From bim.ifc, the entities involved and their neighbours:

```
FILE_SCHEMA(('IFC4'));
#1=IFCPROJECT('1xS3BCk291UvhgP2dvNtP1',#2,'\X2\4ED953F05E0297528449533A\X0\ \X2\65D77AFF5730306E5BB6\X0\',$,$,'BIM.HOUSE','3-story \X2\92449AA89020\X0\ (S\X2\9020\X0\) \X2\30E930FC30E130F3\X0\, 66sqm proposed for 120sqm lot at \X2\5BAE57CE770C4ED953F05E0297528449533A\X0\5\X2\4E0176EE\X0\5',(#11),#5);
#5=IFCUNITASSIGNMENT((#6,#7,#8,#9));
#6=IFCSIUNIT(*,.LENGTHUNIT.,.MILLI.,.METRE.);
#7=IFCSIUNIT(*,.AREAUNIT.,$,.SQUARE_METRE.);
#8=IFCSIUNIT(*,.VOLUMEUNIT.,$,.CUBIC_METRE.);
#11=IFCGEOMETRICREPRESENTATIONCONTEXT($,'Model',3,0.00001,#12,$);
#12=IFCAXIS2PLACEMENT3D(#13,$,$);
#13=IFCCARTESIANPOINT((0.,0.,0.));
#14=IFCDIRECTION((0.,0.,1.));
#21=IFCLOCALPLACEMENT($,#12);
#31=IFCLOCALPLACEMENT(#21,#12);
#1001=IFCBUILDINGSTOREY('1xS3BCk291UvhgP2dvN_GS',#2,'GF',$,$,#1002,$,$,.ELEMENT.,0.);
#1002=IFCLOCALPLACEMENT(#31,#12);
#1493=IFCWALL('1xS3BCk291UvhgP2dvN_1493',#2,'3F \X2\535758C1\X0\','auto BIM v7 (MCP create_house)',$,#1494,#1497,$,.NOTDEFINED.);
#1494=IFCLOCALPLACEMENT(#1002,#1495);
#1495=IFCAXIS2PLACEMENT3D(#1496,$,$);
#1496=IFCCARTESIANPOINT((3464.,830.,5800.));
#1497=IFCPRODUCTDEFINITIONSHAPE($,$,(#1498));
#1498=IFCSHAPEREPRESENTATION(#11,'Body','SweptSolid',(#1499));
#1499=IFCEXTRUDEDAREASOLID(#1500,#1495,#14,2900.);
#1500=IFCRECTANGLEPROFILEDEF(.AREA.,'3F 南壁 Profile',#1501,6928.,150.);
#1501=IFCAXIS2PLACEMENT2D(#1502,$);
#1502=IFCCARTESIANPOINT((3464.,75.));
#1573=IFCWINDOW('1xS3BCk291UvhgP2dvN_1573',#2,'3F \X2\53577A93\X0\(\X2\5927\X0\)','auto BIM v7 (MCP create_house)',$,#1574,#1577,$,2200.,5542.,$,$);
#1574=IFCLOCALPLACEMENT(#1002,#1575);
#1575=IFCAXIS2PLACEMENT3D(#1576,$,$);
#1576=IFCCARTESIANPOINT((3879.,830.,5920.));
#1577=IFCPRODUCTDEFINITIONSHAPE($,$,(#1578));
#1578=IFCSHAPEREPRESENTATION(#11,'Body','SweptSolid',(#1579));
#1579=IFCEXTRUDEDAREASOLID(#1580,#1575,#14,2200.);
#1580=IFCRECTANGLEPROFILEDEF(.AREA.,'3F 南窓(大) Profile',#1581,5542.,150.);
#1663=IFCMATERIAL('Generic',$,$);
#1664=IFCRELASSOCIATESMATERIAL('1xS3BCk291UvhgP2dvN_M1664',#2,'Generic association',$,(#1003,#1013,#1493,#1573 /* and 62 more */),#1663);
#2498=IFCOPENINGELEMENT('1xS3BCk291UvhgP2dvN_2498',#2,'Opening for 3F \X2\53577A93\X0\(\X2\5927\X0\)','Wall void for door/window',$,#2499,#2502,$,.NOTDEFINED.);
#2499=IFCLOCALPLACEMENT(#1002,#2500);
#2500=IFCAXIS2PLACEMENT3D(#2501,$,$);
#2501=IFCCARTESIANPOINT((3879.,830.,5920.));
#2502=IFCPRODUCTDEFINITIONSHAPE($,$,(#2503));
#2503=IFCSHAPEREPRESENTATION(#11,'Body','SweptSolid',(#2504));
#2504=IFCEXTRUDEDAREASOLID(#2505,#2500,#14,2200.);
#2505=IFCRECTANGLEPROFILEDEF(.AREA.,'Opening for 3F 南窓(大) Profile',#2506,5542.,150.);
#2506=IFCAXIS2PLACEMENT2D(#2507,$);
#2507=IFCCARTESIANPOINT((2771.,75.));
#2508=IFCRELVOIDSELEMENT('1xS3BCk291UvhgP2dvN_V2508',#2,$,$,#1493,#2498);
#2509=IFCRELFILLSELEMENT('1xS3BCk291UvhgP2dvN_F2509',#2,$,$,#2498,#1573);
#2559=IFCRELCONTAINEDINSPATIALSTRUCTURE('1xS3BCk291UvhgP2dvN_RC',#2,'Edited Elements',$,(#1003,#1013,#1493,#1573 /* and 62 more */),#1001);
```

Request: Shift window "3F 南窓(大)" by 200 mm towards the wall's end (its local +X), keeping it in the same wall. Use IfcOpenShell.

```python
import ifcopenshell
import ifcopenshell.api.geometry
import ifcopenshell.util.placement
import ifcopenshell.util.unit

model = ifcopenshell.open("bim.ifc")
unit_scale = ifcopenshell.util.unit.calculate_unit_scale(model)

window = model.by_guid("1xS3BCk291UvhgP2dvN_1573")
opening = window.FillsVoids[0].RelatingOpeningElement
wall = opening.VoidsElements[0].RelatingBuildingElement

wall_matrix = ifcopenshell.util.placement.get_local_placement(wall.ObjectPlacement)
shift = wall_matrix[:3, 0] * 0.2 / unit_scale
before = ifcopenshell.util.placement.get_local_placement(window.ObjectPlacement)[:3, 3].copy()

# The window is not placed relative to its opening, so move both.
for product in (opening, window):
    matrix = ifcopenshell.util.placement.get_local_placement(product.ObjectPlacement)
    matrix[:3, 3] += shift
    ifcopenshell.api.geometry.edit_object_placement(model, product=product, matrix=matrix, is_si=False)

after = ifcopenshell.util.placement.get_local_placement(window.ObjectPlacement)[:3, 3]
print("window moved by", (after - before).round(3) + 0.0)

model.write("bim_v2.ifc")
```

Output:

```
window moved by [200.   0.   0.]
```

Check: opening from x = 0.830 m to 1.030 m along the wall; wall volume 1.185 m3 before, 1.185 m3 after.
